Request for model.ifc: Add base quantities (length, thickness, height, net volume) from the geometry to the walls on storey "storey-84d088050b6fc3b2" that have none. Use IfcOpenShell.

First a look at what the model holds.

```python
import ifcopenshell
import ifcopenshell.util.element
import ifcopenshell.util.unit

model = ifcopenshell.open("model.ifc")
print(model.schema)
for unit_type in ("LENGTHUNIT", "AREAUNIT", "VOLUMEUNIT"):
    print(unit_type, ifcopenshell.util.unit.calculate_unit_scale(model, unit_type))
storey = next(s for s in model.by_type("IfcBuildingStorey") if s.Name == "storey-84d088050b6fc3b2")
walls = [e for e in ifcopenshell.util.element.get_decomposition(storey) if e.is_a("IfcWall")]
for e in sorted(walls, key=lambda e: e.id()):
    print(e.id(), e.is_a(), e.Name, list(ifcopenshell.util.element.get_psets(e, qtos_only=True)), sep=" | ")
```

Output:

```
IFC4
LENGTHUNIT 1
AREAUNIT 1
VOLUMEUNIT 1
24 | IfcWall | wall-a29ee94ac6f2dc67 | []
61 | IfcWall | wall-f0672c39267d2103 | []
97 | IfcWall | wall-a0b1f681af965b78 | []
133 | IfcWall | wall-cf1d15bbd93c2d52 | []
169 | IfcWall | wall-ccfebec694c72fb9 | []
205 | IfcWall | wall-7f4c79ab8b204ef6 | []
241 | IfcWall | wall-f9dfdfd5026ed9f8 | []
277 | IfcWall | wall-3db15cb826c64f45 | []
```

```python
import ifcopenshell
import ifcopenshell.api.pset
import ifcopenshell.geom
import ifcopenshell.util.element
import ifcopenshell.util.shape
import ifcopenshell.util.unit

model = ifcopenshell.open("model.ifc")
unit_scale = ifcopenshell.util.unit.calculate_unit_scale(model)
volume_scale = ifcopenshell.util.unit.calculate_unit_scale(model, "VOLUMEUNIT")
settings = ifcopenshell.geom.settings()

storey = next(s for s in model.by_type("IfcBuildingStorey") if s.Name == "storey-84d088050b6fc3b2")
walls = [e for e in ifcopenshell.util.element.get_decomposition(storey) if e.is_a("IfcWall")]

for e in sorted(walls, key=lambda e: e.id()):
    if ifcopenshell.util.element.get_psets(e, qtos_only=True, should_inherit=False):
        continue
    # Geometry comes back in metres, in the element's own axes.
    shape = ifcopenshell.geom.create_shape(settings, e)
    values = {
        "Length": ifcopenshell.util.shape.get_x(shape.geometry) / unit_scale,
        "Width": ifcopenshell.util.shape.get_y(shape.geometry) / unit_scale,
        "Height": ifcopenshell.util.shape.get_z(shape.geometry) / unit_scale,
        "NetVolume": ifcopenshell.util.shape.get_volume(shape.geometry) / volume_scale,
    }
    qto = ifcopenshell.api.pset.add_qto(model, product=e, name="Qto_WallBaseQuantities")
    ifcopenshell.api.pset.edit_qto(model, qto=qto, properties=values)
    print(e.id(), {k: round(v, 3) for k, v in values.items()})

model.write("model-out.ifc")
```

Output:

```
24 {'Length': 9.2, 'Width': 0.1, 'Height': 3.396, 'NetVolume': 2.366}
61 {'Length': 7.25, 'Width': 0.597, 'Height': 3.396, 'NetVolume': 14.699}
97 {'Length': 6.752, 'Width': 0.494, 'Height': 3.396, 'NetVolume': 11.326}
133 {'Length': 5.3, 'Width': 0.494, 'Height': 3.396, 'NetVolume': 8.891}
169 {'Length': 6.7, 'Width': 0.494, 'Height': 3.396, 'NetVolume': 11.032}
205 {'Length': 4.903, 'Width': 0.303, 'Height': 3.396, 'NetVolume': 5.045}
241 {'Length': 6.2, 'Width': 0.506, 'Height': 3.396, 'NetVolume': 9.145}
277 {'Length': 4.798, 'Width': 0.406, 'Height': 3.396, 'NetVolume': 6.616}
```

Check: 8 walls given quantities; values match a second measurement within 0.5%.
